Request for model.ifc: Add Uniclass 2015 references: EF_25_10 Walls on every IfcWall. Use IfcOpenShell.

First a look at what the model holds.

```python
import ifcopenshell

model = ifcopenshell.open("model.ifc")
print(model.schema)
print("classifications:", [c.Name for c in model.by_type("IfcClassification")])
for ifc_class in ("IfcDoor", "IfcRoof", "IfcStair", "IfcWall", "IfcWindow"):
    print(ifc_class, len(model.by_type(ifc_class)))
```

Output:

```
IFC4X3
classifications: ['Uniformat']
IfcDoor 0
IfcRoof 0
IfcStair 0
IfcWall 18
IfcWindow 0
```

```python
import ifcopenshell
import ifcopenshell.api.classification

model = ifcopenshell.open("model.ifc")

system = ifcopenshell.api.classification.add_classification(model, classification="Uniclass 2015")

codes = {
    "IfcWall": ("EF_25_10", "Walls"),
}
for ifc_class, (code, name) in codes.items():
    products = model.by_type(ifc_class)
    ifcopenshell.api.classification.add_reference(
        model, products=products, classification=system, identification=code, name=name
    )
    print(code, len(products))

model.write("model_v2.ifc")
```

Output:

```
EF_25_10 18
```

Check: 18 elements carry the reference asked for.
